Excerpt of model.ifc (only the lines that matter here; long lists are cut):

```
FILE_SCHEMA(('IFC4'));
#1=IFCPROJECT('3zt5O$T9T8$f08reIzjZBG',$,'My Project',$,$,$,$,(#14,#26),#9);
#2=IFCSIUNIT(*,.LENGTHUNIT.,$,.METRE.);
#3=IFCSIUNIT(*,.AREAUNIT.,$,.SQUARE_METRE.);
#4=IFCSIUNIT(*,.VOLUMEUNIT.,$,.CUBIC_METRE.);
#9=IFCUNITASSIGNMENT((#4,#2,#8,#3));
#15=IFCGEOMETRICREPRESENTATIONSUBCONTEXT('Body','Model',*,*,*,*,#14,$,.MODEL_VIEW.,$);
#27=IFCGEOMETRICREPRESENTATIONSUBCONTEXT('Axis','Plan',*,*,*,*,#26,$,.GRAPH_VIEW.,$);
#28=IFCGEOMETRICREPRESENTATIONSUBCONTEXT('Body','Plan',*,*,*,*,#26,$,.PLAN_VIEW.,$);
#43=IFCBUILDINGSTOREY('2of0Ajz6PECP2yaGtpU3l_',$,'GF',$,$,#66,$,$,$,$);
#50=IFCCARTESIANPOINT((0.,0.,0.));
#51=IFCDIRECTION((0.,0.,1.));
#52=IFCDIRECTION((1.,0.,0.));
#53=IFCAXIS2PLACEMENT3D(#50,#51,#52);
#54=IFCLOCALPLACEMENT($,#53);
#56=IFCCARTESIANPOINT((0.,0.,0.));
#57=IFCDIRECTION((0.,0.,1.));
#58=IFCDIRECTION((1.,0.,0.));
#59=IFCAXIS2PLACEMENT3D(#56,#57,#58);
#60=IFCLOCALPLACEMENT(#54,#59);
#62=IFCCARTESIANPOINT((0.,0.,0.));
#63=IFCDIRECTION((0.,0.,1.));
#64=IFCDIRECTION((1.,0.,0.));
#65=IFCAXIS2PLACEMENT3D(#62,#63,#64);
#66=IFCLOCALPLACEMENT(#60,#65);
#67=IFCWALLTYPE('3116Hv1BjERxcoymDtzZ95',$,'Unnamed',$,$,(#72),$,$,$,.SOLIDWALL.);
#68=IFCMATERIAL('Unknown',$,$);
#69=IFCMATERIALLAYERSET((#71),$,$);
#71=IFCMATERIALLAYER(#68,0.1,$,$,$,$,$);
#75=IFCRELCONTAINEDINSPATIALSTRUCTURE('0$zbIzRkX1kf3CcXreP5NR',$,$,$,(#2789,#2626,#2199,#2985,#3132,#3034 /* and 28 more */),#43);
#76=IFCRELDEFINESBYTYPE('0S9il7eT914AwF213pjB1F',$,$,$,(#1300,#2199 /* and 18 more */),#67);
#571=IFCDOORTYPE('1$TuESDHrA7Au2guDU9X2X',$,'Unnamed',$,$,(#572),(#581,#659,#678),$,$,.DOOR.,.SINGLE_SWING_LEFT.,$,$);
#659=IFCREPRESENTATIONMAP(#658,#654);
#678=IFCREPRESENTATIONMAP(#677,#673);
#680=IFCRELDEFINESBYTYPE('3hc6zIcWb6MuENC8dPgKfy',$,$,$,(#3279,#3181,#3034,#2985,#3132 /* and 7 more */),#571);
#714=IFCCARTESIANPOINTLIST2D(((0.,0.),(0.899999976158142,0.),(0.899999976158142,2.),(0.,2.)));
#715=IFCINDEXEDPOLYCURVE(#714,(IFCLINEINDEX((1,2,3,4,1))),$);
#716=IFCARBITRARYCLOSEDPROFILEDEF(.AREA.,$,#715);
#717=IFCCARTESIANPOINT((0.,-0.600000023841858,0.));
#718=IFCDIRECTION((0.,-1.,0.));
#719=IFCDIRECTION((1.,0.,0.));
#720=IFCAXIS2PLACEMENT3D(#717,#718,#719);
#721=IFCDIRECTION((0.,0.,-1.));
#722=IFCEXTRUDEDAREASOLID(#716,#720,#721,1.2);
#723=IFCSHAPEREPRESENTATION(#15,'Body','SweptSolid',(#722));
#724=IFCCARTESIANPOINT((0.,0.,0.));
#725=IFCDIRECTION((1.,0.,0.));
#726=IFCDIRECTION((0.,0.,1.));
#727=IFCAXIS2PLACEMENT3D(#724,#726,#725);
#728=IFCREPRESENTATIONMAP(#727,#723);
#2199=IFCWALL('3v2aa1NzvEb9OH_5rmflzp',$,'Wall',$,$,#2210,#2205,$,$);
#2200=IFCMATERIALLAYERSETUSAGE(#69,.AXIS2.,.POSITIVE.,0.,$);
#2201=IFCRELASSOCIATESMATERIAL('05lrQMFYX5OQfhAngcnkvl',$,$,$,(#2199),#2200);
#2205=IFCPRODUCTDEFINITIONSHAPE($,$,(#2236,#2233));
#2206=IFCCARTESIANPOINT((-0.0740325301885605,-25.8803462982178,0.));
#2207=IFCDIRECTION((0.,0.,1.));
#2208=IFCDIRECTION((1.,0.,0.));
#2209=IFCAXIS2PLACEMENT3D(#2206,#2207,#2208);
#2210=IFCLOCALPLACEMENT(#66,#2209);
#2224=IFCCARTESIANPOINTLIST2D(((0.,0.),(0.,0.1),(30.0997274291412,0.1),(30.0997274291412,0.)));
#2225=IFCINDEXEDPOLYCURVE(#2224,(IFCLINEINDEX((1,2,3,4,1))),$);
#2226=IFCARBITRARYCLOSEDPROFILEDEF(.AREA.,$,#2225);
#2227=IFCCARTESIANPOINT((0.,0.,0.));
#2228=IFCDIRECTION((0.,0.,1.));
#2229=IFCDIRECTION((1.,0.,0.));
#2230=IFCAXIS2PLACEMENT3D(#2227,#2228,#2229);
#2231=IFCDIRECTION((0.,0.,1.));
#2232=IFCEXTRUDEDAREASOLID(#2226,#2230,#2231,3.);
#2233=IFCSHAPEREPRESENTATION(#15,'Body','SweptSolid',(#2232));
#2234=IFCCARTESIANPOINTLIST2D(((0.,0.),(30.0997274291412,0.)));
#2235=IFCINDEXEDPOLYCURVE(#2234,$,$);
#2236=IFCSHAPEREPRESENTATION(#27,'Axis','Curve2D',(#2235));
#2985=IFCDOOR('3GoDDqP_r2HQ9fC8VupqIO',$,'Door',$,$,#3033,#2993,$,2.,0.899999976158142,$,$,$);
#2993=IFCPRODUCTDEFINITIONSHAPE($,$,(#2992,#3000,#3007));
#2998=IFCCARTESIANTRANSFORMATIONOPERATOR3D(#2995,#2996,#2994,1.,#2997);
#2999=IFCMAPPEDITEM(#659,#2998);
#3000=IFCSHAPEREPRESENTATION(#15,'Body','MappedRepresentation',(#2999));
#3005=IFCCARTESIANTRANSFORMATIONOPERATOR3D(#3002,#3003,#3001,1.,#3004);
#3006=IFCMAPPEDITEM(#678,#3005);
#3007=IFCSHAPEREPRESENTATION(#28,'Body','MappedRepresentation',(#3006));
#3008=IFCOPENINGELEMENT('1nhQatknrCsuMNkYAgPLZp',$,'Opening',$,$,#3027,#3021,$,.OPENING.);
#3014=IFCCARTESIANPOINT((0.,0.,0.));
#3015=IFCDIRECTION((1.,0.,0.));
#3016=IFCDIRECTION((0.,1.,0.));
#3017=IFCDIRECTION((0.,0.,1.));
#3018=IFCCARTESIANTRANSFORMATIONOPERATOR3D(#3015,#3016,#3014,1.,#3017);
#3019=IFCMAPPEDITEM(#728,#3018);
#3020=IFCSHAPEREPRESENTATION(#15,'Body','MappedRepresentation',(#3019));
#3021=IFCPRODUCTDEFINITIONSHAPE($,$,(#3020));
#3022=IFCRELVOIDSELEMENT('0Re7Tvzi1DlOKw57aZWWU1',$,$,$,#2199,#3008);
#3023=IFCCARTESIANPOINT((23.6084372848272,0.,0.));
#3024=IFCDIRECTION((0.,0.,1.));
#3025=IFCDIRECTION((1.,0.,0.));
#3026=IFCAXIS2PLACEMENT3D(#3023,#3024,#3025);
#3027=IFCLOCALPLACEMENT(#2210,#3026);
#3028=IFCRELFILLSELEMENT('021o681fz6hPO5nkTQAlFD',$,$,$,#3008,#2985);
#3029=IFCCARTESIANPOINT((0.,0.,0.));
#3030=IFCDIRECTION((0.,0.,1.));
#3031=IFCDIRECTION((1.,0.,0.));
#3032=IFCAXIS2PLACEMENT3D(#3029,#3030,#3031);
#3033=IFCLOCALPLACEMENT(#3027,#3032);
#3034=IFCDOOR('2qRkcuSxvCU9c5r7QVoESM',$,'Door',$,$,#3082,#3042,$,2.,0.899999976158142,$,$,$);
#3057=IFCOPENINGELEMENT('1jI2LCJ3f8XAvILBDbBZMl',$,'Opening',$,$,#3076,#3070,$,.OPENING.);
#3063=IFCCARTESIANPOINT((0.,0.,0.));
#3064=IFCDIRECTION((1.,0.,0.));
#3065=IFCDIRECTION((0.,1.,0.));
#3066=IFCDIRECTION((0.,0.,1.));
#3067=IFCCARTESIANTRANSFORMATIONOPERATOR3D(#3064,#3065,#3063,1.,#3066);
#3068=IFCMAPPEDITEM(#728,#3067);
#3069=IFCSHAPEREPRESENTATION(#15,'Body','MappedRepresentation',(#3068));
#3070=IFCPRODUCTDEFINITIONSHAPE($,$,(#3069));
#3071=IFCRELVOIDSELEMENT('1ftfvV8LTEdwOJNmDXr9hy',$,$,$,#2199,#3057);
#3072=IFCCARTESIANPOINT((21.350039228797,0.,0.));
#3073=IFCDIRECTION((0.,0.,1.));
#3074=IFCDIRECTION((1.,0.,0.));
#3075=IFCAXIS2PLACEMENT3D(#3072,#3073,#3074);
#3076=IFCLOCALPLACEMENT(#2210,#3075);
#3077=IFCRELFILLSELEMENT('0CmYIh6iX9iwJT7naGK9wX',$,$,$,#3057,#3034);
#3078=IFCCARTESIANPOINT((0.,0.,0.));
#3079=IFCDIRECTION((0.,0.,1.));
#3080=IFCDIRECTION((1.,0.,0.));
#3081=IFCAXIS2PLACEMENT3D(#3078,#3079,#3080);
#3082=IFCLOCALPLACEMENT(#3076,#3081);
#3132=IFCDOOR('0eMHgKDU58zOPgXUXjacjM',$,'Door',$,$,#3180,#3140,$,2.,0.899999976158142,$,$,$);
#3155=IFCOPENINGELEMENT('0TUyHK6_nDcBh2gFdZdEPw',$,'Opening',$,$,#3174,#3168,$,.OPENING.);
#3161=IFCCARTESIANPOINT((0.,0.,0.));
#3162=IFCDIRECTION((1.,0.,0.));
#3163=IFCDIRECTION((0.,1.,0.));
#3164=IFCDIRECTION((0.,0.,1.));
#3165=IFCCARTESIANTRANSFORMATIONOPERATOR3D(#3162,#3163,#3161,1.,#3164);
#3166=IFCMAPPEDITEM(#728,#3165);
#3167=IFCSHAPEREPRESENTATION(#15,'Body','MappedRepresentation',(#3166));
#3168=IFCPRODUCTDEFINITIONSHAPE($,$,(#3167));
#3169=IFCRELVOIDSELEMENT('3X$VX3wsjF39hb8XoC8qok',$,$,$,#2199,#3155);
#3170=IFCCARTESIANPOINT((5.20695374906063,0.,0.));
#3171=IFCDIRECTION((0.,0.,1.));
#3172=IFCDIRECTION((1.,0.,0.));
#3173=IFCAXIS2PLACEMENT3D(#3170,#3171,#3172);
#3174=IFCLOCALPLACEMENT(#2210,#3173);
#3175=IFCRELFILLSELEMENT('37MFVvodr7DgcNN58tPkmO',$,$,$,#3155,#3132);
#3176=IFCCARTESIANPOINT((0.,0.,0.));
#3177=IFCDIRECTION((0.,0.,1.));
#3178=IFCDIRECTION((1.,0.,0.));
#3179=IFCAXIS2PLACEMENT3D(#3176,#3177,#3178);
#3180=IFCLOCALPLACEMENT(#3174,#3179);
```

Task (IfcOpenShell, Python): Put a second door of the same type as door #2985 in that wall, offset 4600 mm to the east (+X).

```python
import ifcopenshell
import ifcopenshell.api.feature
import ifcopenshell.api.geometry
import ifcopenshell.api.root
import ifcopenshell.geom
import ifcopenshell.util.element
import ifcopenshell.util.placement
import ifcopenshell.util.shape
import ifcopenshell.util.unit

model = ifcopenshell.open("model.ifc")
unit_scale = ifcopenshell.util.unit.calculate_unit_scale(model)
settings = ifcopenshell.geom.settings()


def volume(element):
    """Net volume in cubic metres, openings subtracted."""
    shape = ifcopenshell.geom.create_shape(settings, element)
    return ifcopenshell.util.shape.get_volume(shape.geometry)


door = model.by_guid("3GoDDqP_r2HQ9fC8VupqIO")
opening = door.FillsVoids[0].RelatingOpeningElement
wall = opening.VoidsElements[0].RelatingBuildingElement
before = volume(wall)
shift = ifcopenshell.util.placement.get_local_placement(wall.ObjectPlacement)[:3, 0] * 4.6 / unit_scale

# copy_class copies the void relationship, type, container and properties, but no geometry.
new_opening = ifcopenshell.api.root.copy_class(model, product=opening)
new_opening.Representation = ifcopenshell.util.element.copy_deep(
    model, opening.Representation, exclude=["IfcGeometricRepresentationContext", "IfcRepresentationMap"]
)
new_door = ifcopenshell.api.root.copy_class(model, product=door)
new_door.Representation = ifcopenshell.util.element.copy_deep(
    model, door.Representation, exclude=["IfcGeometricRepresentationContext", "IfcRepresentationMap"]
)
ifcopenshell.api.feature.add_filling(model, opening=new_opening, element=new_door)

for old, new in ((opening, new_opening), (door, new_door)):
    matrix = ifcopenshell.util.placement.get_local_placement(old.ObjectPlacement)
    matrix[:3, 3] += shift
    ifcopenshell.api.geometry.edit_object_placement(model, product=new, matrix=matrix, is_si=False)

after = volume(wall)

print(f"wall volume {before:.3f} -> {after:.3f} m3")

model.write("model_v2.ifc")
```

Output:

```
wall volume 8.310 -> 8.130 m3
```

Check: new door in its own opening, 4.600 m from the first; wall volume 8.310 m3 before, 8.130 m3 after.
